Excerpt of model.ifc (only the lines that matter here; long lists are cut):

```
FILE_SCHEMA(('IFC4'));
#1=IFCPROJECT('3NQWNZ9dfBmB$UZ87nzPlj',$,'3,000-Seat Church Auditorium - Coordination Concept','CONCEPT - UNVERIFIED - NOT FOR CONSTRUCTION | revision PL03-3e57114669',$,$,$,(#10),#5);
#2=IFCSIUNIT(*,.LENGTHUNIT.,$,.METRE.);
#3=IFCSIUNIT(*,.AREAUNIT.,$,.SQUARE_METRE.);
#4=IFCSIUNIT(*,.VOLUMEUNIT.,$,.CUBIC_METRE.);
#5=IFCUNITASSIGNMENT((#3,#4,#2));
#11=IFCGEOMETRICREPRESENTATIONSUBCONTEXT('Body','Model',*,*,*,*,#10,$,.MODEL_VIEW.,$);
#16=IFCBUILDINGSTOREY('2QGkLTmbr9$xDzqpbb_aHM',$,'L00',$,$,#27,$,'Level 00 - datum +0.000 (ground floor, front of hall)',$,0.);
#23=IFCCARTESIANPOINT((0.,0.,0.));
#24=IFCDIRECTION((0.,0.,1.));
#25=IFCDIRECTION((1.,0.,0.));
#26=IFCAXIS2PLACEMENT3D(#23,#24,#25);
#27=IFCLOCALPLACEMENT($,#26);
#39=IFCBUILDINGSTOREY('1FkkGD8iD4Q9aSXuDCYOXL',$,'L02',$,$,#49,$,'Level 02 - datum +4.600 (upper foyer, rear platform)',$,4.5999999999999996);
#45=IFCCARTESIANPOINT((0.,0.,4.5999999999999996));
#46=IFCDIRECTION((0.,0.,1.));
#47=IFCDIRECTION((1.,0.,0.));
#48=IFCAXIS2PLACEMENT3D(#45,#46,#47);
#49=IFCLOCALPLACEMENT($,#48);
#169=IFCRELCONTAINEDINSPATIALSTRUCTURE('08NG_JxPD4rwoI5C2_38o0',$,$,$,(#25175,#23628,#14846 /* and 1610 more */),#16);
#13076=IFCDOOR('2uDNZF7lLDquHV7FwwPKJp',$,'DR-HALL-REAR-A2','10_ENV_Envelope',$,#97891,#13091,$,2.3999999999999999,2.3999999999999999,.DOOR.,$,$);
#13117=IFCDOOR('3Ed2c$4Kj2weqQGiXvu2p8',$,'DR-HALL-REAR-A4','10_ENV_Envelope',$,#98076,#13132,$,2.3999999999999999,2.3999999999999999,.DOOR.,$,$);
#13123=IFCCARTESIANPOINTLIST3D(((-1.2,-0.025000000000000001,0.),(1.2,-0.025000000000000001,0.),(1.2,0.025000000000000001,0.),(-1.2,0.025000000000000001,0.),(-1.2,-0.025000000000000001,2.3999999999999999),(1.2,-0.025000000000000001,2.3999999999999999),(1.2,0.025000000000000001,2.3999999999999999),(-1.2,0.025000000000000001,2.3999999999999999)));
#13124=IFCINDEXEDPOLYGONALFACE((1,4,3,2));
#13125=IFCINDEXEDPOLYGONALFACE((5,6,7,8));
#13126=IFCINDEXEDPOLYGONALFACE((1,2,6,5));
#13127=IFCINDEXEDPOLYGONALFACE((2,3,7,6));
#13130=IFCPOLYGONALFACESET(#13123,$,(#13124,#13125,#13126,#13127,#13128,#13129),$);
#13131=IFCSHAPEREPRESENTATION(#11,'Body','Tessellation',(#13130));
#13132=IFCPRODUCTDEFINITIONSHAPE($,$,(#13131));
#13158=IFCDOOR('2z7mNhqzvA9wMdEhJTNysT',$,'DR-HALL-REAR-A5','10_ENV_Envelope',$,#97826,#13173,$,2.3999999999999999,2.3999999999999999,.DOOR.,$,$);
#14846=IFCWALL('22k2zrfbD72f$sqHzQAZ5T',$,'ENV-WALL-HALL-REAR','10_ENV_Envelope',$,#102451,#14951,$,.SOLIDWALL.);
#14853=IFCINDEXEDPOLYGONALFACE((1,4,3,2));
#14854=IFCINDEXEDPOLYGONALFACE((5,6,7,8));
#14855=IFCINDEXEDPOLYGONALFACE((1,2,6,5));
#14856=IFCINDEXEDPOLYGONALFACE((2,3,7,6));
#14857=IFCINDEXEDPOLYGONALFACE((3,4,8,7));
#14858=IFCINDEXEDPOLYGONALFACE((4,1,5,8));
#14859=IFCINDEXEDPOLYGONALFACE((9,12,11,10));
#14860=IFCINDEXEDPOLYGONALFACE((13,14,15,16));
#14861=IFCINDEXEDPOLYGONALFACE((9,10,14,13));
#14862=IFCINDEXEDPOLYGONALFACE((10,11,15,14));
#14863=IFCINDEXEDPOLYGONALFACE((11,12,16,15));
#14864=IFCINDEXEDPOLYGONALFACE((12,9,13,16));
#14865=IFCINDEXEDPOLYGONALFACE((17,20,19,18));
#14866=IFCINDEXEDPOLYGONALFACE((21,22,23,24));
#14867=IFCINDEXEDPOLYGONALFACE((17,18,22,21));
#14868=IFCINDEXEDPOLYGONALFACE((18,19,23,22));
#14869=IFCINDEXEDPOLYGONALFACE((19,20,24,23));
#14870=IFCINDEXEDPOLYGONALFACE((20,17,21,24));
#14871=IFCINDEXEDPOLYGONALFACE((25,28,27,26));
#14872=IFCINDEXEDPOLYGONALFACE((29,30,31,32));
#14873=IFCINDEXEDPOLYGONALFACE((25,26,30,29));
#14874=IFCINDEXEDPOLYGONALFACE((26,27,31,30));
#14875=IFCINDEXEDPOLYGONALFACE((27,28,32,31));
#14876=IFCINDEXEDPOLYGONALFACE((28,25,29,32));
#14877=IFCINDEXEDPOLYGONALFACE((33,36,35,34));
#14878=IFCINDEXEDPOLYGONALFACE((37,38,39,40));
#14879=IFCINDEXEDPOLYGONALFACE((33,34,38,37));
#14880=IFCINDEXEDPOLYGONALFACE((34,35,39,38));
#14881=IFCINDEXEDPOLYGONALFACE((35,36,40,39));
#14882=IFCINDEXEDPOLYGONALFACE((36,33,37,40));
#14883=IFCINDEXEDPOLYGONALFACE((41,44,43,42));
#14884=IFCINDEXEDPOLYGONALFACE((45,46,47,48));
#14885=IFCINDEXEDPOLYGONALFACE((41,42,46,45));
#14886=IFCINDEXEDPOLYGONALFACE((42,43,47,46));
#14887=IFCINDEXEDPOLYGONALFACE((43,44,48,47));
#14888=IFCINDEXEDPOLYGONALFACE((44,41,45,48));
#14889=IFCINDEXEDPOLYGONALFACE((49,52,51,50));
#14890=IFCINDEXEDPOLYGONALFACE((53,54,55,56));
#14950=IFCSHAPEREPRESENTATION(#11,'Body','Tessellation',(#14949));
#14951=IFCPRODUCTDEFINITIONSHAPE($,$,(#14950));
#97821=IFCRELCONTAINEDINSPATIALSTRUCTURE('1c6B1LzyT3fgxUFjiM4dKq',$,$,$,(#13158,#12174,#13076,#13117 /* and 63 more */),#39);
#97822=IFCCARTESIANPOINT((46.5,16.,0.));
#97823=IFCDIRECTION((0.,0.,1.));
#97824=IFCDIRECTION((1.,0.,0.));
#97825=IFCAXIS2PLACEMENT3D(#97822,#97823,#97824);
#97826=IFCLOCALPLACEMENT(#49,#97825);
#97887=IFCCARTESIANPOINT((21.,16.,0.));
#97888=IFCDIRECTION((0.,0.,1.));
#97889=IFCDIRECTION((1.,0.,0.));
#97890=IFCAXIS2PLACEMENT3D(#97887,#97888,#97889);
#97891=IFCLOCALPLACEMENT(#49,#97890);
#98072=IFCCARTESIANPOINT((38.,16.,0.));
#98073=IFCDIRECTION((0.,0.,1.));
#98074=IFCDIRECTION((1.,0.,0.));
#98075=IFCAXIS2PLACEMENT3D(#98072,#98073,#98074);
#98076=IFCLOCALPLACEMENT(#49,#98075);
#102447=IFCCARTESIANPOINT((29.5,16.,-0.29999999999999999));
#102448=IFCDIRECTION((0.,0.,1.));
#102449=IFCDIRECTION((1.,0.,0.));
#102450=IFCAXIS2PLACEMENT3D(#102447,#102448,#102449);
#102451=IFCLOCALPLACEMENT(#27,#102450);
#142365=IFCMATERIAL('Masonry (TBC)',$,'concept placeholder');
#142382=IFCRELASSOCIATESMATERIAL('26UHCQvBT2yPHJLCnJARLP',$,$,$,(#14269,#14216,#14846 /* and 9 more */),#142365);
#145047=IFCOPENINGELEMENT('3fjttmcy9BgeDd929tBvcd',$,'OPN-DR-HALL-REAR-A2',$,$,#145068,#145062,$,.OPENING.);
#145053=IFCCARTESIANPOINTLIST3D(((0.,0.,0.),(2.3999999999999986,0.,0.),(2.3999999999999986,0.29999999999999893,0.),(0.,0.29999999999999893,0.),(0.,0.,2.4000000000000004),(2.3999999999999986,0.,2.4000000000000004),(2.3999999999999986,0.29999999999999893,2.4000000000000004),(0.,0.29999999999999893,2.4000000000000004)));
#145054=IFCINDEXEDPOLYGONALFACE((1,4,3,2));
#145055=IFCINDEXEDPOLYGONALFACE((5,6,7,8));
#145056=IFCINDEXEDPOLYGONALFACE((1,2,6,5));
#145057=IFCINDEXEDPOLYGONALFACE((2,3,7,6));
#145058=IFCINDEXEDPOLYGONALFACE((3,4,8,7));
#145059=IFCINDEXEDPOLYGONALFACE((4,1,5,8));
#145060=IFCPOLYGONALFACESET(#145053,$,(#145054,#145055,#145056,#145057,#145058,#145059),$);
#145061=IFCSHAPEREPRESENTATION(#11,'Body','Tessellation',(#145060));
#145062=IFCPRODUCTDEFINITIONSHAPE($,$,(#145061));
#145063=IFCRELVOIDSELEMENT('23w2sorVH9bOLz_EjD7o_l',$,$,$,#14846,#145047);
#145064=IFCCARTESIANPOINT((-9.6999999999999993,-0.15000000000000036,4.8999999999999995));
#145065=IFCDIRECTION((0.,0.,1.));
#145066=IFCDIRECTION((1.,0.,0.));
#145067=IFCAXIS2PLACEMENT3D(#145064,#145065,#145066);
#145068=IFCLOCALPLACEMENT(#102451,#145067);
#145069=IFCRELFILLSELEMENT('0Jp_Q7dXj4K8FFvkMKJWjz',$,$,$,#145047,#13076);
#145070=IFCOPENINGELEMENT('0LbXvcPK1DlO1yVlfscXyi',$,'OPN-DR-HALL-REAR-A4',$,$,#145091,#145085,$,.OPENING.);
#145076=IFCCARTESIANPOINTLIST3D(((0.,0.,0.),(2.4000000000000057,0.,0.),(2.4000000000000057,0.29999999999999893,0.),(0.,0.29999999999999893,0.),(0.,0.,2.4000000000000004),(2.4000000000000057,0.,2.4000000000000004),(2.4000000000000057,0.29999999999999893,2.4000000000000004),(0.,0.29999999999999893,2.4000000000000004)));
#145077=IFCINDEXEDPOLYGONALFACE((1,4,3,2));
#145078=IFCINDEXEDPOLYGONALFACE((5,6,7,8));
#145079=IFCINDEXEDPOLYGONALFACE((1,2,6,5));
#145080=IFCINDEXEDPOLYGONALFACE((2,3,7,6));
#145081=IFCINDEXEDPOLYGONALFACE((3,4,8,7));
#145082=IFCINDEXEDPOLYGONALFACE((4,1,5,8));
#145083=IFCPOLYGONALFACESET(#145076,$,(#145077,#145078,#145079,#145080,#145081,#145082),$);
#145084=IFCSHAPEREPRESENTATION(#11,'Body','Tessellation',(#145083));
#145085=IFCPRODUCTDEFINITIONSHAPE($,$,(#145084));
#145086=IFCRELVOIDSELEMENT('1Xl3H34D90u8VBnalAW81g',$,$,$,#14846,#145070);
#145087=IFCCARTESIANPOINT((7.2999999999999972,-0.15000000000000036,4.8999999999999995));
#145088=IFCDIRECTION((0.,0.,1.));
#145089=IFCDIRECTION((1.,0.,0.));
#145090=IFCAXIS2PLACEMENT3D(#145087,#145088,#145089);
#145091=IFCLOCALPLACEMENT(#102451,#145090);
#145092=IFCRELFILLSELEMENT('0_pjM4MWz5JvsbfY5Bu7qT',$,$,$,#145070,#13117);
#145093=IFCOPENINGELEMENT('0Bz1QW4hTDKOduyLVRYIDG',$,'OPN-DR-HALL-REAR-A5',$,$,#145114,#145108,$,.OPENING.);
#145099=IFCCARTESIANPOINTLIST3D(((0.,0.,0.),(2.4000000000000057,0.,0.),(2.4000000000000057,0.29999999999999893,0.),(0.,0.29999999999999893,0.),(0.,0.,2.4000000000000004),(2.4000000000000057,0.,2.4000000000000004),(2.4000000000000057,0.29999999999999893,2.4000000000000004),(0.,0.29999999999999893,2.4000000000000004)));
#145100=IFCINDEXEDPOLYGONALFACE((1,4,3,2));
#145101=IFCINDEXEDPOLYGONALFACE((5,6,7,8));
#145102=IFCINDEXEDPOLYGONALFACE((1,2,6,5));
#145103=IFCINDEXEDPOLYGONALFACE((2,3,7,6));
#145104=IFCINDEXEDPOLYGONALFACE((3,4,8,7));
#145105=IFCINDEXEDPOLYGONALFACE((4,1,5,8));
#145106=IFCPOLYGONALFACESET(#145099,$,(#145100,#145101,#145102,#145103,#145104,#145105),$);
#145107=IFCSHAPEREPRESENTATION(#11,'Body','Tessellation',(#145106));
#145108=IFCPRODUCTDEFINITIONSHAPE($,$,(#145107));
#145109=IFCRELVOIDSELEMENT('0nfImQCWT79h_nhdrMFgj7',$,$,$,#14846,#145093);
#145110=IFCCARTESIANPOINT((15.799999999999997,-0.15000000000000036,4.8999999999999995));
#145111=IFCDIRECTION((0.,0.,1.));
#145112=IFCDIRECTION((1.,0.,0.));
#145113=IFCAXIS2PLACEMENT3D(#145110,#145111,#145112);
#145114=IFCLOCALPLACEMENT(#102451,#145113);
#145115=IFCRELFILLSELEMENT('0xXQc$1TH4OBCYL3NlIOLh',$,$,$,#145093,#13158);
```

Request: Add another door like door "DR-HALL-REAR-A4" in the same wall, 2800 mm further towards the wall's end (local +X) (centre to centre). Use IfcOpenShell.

```python
import ifcopenshell
import ifcopenshell.api.feature
import ifcopenshell.api.geometry
import ifcopenshell.api.root
import ifcopenshell.geom
import ifcopenshell.util.element
import ifcopenshell.util.placement
import ifcopenshell.util.shape
import ifcopenshell.util.unit

model = ifcopenshell.open("model.ifc")
unit_scale = ifcopenshell.util.unit.calculate_unit_scale(model)
settings = ifcopenshell.geom.settings()


def volume(element):
    """Net volume in cubic metres, openings subtracted."""
    shape = ifcopenshell.geom.create_shape(settings, element)
    return ifcopenshell.util.shape.get_volume(shape.geometry)


door = model.by_guid("3Ed2c$4Kj2weqQGiXvu2p8")
opening = door.FillsVoids[0].RelatingOpeningElement
wall = opening.VoidsElements[0].RelatingBuildingElement
before = volume(wall)
shift = ifcopenshell.util.placement.get_local_placement(wall.ObjectPlacement)[:3, 0] * 2.8 / unit_scale

# copy_class copies the void relationship, type, container and properties, but no geometry.
new_opening = ifcopenshell.api.root.copy_class(model, product=opening)
new_opening.Representation = ifcopenshell.util.element.copy_deep(
    model, opening.Representation, exclude=["IfcGeometricRepresentationContext", "IfcRepresentationMap"]
)
new_door = ifcopenshell.api.root.copy_class(model, product=door)
new_door.Representation = ifcopenshell.util.element.copy_deep(
    model, door.Representation, exclude=["IfcGeometricRepresentationContext", "IfcRepresentationMap"]
)
ifcopenshell.api.feature.add_filling(model, opening=new_opening, element=new_door)

for old, new in ((opening, new_opening), (door, new_door)):
    matrix = ifcopenshell.util.placement.get_local_placement(old.ObjectPlacement)
    matrix[:3, 3] += shift
    ifcopenshell.api.geometry.edit_object_placement(model, product=new, matrix=matrix, is_si=False)

after = volume(wall)

print(f"wall volume {before:.3f} -> {after:.3f} m3")

model.write("model-out.ifc")
```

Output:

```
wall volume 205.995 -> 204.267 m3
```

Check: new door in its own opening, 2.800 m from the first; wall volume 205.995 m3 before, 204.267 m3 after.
